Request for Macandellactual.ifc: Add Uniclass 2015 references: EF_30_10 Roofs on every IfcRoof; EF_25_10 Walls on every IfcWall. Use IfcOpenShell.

First a look at what the model holds.

```python
import ifcopenshell

model = ifcopenshell.open("Macandellactual.ifc")
print(model.schema)
print("classifications:", [c.Name for c in model.by_type("IfcClassification")])
for ifc_class in ("IfcDoor", "IfcRoof", "IfcStair", "IfcWall", "IfcWindow"):
    print(ifc_class, len(model.by_type(ifc_class)))
```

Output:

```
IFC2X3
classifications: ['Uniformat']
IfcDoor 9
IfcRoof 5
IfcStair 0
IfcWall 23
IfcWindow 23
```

```python
import ifcopenshell
import ifcopenshell.api.classification

model = ifcopenshell.open("Macandellactual.ifc")

# IFC2X3 requires Source and Edition and has no link from the project to the system.
system = model.create_entity("IfcClassification", Source="NBS", Edition="2015", Name="Uniclass 2015")

codes = {
    "IfcRoof": ("EF_30_10", "Roofs"),
    "IfcWall": ("EF_25_10", "Walls"),
}
for ifc_class, (code, name) in codes.items():
    products = model.by_type(ifc_class)
    ifcopenshell.api.classification.add_reference(
        model, products=products, classification=system, identification=code, name=name
    )
    print(code, len(products))

model.write("Macandellactual_v2.ifc")
```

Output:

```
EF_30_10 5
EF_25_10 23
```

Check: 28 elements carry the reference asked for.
